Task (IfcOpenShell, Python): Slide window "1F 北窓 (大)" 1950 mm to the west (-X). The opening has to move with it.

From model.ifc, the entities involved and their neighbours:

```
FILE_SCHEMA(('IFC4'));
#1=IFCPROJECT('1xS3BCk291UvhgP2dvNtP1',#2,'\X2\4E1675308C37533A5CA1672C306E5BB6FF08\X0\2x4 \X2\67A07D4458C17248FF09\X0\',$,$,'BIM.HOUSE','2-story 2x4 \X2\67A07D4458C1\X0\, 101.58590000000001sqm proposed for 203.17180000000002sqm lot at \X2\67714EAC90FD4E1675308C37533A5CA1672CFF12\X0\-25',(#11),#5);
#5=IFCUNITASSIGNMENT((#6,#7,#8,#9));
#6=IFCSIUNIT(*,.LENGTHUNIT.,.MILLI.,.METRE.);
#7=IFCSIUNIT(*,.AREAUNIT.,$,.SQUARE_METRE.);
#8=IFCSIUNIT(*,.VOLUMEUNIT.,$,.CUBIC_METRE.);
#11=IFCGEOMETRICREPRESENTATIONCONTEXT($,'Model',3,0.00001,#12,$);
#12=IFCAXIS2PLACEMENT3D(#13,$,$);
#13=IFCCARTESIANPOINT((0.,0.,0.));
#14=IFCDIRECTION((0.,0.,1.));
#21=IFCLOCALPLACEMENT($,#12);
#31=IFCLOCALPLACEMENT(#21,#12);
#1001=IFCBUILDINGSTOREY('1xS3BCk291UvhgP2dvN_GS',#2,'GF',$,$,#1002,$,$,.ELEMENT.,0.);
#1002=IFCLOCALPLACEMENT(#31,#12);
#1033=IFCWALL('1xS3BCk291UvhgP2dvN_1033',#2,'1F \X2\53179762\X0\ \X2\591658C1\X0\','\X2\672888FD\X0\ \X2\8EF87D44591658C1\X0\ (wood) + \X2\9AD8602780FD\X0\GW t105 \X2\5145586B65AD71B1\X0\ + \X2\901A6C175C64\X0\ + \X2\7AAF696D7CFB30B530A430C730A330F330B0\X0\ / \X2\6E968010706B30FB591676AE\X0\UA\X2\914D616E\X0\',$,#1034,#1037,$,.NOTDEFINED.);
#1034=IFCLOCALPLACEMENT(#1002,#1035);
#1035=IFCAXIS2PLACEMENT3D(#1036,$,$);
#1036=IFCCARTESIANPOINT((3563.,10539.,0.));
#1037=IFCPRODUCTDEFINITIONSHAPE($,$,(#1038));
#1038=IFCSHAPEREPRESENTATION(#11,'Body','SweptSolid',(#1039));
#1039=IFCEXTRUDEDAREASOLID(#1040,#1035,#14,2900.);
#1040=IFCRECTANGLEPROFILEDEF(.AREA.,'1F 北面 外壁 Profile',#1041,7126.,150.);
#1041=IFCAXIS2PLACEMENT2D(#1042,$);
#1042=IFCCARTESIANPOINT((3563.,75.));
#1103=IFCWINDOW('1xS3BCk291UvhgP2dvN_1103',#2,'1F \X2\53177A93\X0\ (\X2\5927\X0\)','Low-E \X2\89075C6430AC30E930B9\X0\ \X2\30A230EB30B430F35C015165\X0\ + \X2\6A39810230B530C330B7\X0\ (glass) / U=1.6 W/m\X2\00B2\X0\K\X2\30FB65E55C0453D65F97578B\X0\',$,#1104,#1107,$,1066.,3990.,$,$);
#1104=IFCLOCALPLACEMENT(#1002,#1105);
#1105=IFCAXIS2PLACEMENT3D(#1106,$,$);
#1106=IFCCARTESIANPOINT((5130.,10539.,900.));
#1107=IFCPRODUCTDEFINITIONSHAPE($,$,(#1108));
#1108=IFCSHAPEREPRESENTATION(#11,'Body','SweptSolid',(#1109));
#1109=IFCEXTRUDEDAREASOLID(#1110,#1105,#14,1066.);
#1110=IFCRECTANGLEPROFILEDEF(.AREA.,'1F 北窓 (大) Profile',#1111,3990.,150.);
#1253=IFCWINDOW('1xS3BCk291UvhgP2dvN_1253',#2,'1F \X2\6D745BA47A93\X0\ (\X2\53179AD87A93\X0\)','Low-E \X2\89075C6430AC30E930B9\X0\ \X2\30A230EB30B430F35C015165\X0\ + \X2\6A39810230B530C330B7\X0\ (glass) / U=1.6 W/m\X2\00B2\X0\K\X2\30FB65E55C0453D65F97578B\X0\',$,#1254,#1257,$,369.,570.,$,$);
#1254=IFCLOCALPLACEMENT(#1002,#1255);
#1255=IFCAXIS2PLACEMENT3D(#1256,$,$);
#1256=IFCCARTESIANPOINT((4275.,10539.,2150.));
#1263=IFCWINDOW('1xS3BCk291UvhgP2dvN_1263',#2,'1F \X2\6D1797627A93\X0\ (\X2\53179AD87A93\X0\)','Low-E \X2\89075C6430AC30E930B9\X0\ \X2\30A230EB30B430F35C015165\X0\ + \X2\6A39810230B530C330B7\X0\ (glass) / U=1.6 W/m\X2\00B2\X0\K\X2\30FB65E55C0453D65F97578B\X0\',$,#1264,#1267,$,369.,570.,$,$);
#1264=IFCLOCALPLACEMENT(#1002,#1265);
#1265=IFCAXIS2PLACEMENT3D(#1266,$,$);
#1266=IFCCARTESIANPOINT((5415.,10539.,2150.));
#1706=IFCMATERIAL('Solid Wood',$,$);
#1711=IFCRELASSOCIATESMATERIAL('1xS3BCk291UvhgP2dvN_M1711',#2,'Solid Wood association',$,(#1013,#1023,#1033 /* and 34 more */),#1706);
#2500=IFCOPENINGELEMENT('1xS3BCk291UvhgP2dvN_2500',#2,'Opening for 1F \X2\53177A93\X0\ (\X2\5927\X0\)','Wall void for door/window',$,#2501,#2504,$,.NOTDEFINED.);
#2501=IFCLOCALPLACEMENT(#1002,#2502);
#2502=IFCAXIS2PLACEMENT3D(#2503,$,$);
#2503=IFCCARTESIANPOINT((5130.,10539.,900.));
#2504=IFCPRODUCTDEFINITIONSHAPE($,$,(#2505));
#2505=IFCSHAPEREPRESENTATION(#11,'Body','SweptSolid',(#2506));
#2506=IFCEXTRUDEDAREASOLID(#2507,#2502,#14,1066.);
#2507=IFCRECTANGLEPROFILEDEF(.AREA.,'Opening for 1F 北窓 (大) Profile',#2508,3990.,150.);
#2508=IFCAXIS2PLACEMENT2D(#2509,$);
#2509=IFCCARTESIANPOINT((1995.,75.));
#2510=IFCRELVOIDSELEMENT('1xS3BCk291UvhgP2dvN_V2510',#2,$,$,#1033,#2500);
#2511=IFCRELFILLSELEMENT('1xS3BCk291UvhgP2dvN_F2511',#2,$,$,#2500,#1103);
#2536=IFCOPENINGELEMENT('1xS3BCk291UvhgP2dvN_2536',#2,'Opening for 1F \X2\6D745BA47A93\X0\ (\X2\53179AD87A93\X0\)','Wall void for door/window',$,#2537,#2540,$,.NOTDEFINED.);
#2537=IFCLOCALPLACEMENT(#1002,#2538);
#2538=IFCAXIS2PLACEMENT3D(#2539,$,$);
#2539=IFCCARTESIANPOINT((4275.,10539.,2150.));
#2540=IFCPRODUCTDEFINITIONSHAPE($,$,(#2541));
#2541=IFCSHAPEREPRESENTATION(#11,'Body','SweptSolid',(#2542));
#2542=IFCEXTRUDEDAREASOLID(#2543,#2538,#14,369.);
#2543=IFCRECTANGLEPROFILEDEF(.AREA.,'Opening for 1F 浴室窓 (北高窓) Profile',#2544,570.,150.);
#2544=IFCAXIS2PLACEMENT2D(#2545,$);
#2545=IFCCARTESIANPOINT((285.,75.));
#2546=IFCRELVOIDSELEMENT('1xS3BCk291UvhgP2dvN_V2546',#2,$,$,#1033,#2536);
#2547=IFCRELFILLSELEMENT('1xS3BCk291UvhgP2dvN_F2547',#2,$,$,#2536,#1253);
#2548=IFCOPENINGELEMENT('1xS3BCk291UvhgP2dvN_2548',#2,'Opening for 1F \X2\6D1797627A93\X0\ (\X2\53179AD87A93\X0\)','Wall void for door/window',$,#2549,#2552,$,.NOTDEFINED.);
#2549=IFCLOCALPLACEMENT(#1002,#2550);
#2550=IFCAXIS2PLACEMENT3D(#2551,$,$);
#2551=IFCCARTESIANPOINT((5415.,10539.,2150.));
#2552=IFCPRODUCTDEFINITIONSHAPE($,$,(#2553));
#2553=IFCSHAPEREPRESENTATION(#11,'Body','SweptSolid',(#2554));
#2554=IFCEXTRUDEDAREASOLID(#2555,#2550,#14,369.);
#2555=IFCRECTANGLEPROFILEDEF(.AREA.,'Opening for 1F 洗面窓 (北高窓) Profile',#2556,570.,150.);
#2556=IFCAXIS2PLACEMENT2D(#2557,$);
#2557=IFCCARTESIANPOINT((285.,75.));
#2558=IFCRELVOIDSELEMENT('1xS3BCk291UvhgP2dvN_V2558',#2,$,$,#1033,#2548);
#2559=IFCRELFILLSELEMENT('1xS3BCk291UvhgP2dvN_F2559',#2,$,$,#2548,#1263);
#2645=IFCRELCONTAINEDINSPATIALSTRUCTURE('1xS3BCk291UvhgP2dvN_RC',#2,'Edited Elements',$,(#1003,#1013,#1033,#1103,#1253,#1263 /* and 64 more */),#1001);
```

```python
import ifcopenshell
import ifcopenshell.api.geometry
import ifcopenshell.util.placement

model = ifcopenshell.open("model.ifc")

window = model.by_id(1103)
opening = window.FillsVoids[0].RelatingOpeningElement
wall = opening.VoidsElements[0].RelatingBuildingElement

wall_matrix = ifcopenshell.util.placement.get_local_placement(wall.ObjectPlacement)
shift = wall_matrix[:3, 0] * -1950.0
before = ifcopenshell.util.placement.get_local_placement(window.ObjectPlacement)[:3, 3].copy()

# The window is not placed relative to its opening, so move both.
for product in (opening, window):
    matrix = ifcopenshell.util.placement.get_local_placement(product.ObjectPlacement)
    matrix[:3, 3] += shift
    ifcopenshell.api.geometry.edit_object_placement(model, product=product, matrix=matrix, is_si=False)

after = ifcopenshell.util.placement.get_local_placement(window.ObjectPlacement)[:3, 3]
print("window moved by", (after - before).round(3) + 0.0)

model.write("model-out.ifc")
```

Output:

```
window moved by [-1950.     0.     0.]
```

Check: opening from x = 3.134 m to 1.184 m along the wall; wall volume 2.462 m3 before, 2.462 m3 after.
